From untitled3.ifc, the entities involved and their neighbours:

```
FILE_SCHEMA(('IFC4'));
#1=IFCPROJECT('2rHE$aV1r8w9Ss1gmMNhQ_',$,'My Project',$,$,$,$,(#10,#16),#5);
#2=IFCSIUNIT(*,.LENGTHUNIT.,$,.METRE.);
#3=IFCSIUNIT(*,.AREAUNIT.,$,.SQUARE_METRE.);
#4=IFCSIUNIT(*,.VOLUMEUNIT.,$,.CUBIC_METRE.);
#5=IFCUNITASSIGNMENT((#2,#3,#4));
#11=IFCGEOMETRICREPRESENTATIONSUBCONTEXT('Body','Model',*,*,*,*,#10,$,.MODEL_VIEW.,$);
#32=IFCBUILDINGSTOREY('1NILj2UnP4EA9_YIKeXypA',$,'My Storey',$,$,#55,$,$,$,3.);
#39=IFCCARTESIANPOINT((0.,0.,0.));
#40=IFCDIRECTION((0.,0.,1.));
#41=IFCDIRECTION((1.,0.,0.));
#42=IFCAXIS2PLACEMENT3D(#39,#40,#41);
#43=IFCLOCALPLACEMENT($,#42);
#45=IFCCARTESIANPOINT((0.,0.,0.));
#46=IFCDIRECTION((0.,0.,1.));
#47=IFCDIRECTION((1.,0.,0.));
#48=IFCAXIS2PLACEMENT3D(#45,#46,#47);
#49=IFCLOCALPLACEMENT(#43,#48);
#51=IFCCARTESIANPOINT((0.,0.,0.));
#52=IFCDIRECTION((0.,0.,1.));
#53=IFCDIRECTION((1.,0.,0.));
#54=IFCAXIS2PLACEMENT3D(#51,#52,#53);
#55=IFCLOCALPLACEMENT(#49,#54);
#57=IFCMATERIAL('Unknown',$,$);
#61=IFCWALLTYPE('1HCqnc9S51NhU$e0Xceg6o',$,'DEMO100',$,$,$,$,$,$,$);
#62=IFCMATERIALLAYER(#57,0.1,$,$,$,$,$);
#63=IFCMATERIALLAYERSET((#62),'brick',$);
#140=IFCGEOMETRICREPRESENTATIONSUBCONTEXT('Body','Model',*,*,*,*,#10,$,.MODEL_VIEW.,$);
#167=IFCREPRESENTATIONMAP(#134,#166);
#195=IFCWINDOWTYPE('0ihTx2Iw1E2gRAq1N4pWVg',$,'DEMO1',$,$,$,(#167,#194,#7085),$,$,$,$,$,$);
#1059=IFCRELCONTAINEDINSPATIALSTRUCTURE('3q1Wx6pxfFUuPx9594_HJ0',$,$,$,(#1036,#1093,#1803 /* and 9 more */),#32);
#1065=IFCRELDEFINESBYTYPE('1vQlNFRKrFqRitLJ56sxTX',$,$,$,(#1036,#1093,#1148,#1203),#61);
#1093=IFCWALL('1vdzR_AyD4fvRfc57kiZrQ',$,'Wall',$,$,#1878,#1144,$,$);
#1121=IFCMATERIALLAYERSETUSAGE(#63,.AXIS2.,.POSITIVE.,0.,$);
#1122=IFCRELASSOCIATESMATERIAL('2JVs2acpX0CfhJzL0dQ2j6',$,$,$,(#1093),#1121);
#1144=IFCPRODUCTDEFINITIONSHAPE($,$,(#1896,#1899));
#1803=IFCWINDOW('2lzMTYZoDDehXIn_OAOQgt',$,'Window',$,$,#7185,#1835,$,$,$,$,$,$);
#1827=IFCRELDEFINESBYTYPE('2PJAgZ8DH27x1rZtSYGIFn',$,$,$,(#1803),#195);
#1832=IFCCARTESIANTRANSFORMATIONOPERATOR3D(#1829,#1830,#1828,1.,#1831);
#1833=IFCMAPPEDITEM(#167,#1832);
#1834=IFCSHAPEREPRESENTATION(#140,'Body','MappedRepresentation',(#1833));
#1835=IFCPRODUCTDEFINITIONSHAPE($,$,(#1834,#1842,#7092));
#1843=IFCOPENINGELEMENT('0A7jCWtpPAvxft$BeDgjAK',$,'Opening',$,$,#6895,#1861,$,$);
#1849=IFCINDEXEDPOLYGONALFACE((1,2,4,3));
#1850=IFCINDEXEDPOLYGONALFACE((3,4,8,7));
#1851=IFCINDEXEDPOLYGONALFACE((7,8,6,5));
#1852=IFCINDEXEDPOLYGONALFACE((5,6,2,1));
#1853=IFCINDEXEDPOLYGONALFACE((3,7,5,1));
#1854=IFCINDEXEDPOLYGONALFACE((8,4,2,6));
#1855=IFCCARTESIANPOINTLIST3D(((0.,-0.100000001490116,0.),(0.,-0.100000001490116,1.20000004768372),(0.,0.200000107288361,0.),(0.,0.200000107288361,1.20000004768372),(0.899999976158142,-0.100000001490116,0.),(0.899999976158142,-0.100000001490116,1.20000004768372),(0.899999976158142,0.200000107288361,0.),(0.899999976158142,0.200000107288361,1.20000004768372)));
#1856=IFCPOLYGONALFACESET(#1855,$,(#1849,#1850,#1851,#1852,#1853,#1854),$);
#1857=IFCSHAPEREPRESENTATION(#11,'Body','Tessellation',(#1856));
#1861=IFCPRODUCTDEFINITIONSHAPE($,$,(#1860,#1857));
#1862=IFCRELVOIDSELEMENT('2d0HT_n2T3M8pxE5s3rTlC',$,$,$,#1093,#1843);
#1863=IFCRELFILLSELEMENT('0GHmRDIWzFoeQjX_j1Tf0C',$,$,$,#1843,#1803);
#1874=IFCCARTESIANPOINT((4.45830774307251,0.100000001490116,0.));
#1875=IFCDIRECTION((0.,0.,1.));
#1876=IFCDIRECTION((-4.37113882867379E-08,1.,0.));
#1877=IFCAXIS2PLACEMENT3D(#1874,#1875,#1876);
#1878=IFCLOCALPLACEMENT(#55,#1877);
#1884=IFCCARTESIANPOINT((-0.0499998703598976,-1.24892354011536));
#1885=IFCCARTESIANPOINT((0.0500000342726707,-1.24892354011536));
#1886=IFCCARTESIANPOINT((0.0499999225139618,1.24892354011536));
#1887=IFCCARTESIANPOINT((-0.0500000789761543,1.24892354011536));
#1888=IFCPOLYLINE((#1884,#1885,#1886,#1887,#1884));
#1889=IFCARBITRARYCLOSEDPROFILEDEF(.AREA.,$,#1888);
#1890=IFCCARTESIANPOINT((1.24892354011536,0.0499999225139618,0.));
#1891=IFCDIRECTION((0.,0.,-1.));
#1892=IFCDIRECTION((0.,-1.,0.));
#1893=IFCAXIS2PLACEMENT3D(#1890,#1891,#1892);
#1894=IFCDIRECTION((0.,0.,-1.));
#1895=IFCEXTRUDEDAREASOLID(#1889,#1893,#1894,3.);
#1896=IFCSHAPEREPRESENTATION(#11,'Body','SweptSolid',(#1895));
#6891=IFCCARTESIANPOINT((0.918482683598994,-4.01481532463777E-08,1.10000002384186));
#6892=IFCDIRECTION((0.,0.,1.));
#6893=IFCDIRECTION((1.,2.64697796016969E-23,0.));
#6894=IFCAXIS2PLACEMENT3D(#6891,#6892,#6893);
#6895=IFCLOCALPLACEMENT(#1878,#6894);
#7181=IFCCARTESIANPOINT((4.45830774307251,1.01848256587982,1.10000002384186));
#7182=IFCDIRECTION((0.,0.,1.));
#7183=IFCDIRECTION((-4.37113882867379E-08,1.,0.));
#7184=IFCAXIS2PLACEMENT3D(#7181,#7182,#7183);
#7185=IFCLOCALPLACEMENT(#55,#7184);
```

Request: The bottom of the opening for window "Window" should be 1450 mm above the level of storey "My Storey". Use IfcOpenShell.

```python
import numpy as np
import ifcopenshell
import ifcopenshell.api.geometry
import ifcopenshell.geom
import ifcopenshell.util.element
import ifcopenshell.util.placement
import ifcopenshell.util.shape
import ifcopenshell.util.unit

model = ifcopenshell.open("untitled3.ifc")
unit_scale = ifcopenshell.util.unit.calculate_unit_scale(model)

window = model.by_guid("2lzMTYZoDDehXIn_OAOQgt")
opening = window.FillsVoids[0].RelatingOpeningElement
storey = ifcopenshell.util.element.get_container(window, ifc_class="IfcBuildingStorey")
level = ifcopenshell.util.placement.get_local_placement(storey.ObjectPlacement)[2, 3]

# The opening's origin need not be at the sill, so measure its lowest point.
shape = ifcopenshell.geom.create_shape(ifcopenshell.geom.settings(), opening)
bottom = ifcopenshell.util.shape.get_shape_bottom_elevation(shape, shape.geometry) / unit_scale
dz = level + 1.45 / unit_scale - bottom

shift = np.array([0.0, 0.0, dz])
# The window is not placed relative to its opening, so move both.
for product in (opening, window):
    matrix = ifcopenshell.util.placement.get_local_placement(product.ObjectPlacement)
    matrix[:3, 3] += shift
    ifcopenshell.api.geometry.edit_object_placement(model, product=product, matrix=matrix, is_si=False)

print(f"moved by {dz * unit_scale:+.3f} m")

model.write("untitled3_rev.ifc")
```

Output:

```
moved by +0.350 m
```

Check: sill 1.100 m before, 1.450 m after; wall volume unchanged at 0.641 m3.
